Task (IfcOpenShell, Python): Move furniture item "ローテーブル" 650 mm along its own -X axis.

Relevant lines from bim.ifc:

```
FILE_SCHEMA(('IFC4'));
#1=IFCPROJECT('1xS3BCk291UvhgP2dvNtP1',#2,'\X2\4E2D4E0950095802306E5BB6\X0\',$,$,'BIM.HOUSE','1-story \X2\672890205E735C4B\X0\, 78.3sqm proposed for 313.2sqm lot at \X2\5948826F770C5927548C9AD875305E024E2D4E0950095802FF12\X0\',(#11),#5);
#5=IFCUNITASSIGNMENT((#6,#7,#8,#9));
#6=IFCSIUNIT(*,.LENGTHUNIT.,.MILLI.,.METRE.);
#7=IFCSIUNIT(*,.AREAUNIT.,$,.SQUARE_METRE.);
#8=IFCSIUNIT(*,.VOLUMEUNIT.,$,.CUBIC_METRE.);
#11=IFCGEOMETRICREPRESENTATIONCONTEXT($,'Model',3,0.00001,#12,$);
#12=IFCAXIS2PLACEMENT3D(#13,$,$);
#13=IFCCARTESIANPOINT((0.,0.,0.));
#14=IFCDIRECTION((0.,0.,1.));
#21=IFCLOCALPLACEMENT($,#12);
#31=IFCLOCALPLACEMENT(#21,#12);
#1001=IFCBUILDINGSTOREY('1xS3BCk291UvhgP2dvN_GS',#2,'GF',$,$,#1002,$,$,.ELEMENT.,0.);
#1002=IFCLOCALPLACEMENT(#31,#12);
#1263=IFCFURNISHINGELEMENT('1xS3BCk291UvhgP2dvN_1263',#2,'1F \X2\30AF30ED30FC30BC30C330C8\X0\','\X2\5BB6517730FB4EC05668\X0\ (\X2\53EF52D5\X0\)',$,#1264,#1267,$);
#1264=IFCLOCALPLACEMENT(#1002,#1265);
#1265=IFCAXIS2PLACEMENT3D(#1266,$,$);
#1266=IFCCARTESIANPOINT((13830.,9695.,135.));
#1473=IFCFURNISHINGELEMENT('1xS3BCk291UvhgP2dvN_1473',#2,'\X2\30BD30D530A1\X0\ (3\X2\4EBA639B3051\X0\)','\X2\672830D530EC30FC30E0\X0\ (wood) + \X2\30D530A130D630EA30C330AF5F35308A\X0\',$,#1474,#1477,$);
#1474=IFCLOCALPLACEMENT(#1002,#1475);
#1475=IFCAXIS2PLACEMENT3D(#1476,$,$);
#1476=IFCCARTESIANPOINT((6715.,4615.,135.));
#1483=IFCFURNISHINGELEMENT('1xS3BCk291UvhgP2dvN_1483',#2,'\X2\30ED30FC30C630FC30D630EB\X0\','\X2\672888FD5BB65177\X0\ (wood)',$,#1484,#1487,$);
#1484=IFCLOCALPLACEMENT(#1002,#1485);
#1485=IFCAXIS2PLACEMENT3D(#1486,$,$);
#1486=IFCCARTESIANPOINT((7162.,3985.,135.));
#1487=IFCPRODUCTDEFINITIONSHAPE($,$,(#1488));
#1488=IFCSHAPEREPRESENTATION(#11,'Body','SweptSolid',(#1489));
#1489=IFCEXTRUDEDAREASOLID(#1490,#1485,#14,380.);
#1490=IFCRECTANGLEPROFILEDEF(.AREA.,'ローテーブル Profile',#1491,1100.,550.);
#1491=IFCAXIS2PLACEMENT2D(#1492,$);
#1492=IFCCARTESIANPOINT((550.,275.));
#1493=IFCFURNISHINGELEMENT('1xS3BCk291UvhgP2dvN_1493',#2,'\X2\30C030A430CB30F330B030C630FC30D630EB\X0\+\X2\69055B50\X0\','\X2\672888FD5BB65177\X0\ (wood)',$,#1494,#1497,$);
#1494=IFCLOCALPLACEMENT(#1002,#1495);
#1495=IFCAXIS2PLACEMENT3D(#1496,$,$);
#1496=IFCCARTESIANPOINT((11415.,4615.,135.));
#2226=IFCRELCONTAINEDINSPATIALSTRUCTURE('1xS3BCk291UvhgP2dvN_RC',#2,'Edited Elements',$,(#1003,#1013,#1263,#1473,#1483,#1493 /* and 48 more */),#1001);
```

```python
import ifcopenshell
import ifcopenshell.api.geometry
import ifcopenshell.util.placement
import ifcopenshell.util.unit

model = ifcopenshell.open("bim.ifc")
unit_scale = ifcopenshell.util.unit.calculate_unit_scale(model)

item = model.by_id(1483)
matrix = ifcopenshell.util.placement.get_local_placement(item.ObjectPlacement)
matrix[:3, 3] -= matrix[:3, 0] * 0.65 / unit_scale
ifcopenshell.api.geometry.edit_object_placement(model, product=item, matrix=matrix, is_si=False)

print(ifcopenshell.util.placement.get_local_placement(item.ObjectPlacement).round(3) + 0.0)

model.write("bim_rev.ifc")
```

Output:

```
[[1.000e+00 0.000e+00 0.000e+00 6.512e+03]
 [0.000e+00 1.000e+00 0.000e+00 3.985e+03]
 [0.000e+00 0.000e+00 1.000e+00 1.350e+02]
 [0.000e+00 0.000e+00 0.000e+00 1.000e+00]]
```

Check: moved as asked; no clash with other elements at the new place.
